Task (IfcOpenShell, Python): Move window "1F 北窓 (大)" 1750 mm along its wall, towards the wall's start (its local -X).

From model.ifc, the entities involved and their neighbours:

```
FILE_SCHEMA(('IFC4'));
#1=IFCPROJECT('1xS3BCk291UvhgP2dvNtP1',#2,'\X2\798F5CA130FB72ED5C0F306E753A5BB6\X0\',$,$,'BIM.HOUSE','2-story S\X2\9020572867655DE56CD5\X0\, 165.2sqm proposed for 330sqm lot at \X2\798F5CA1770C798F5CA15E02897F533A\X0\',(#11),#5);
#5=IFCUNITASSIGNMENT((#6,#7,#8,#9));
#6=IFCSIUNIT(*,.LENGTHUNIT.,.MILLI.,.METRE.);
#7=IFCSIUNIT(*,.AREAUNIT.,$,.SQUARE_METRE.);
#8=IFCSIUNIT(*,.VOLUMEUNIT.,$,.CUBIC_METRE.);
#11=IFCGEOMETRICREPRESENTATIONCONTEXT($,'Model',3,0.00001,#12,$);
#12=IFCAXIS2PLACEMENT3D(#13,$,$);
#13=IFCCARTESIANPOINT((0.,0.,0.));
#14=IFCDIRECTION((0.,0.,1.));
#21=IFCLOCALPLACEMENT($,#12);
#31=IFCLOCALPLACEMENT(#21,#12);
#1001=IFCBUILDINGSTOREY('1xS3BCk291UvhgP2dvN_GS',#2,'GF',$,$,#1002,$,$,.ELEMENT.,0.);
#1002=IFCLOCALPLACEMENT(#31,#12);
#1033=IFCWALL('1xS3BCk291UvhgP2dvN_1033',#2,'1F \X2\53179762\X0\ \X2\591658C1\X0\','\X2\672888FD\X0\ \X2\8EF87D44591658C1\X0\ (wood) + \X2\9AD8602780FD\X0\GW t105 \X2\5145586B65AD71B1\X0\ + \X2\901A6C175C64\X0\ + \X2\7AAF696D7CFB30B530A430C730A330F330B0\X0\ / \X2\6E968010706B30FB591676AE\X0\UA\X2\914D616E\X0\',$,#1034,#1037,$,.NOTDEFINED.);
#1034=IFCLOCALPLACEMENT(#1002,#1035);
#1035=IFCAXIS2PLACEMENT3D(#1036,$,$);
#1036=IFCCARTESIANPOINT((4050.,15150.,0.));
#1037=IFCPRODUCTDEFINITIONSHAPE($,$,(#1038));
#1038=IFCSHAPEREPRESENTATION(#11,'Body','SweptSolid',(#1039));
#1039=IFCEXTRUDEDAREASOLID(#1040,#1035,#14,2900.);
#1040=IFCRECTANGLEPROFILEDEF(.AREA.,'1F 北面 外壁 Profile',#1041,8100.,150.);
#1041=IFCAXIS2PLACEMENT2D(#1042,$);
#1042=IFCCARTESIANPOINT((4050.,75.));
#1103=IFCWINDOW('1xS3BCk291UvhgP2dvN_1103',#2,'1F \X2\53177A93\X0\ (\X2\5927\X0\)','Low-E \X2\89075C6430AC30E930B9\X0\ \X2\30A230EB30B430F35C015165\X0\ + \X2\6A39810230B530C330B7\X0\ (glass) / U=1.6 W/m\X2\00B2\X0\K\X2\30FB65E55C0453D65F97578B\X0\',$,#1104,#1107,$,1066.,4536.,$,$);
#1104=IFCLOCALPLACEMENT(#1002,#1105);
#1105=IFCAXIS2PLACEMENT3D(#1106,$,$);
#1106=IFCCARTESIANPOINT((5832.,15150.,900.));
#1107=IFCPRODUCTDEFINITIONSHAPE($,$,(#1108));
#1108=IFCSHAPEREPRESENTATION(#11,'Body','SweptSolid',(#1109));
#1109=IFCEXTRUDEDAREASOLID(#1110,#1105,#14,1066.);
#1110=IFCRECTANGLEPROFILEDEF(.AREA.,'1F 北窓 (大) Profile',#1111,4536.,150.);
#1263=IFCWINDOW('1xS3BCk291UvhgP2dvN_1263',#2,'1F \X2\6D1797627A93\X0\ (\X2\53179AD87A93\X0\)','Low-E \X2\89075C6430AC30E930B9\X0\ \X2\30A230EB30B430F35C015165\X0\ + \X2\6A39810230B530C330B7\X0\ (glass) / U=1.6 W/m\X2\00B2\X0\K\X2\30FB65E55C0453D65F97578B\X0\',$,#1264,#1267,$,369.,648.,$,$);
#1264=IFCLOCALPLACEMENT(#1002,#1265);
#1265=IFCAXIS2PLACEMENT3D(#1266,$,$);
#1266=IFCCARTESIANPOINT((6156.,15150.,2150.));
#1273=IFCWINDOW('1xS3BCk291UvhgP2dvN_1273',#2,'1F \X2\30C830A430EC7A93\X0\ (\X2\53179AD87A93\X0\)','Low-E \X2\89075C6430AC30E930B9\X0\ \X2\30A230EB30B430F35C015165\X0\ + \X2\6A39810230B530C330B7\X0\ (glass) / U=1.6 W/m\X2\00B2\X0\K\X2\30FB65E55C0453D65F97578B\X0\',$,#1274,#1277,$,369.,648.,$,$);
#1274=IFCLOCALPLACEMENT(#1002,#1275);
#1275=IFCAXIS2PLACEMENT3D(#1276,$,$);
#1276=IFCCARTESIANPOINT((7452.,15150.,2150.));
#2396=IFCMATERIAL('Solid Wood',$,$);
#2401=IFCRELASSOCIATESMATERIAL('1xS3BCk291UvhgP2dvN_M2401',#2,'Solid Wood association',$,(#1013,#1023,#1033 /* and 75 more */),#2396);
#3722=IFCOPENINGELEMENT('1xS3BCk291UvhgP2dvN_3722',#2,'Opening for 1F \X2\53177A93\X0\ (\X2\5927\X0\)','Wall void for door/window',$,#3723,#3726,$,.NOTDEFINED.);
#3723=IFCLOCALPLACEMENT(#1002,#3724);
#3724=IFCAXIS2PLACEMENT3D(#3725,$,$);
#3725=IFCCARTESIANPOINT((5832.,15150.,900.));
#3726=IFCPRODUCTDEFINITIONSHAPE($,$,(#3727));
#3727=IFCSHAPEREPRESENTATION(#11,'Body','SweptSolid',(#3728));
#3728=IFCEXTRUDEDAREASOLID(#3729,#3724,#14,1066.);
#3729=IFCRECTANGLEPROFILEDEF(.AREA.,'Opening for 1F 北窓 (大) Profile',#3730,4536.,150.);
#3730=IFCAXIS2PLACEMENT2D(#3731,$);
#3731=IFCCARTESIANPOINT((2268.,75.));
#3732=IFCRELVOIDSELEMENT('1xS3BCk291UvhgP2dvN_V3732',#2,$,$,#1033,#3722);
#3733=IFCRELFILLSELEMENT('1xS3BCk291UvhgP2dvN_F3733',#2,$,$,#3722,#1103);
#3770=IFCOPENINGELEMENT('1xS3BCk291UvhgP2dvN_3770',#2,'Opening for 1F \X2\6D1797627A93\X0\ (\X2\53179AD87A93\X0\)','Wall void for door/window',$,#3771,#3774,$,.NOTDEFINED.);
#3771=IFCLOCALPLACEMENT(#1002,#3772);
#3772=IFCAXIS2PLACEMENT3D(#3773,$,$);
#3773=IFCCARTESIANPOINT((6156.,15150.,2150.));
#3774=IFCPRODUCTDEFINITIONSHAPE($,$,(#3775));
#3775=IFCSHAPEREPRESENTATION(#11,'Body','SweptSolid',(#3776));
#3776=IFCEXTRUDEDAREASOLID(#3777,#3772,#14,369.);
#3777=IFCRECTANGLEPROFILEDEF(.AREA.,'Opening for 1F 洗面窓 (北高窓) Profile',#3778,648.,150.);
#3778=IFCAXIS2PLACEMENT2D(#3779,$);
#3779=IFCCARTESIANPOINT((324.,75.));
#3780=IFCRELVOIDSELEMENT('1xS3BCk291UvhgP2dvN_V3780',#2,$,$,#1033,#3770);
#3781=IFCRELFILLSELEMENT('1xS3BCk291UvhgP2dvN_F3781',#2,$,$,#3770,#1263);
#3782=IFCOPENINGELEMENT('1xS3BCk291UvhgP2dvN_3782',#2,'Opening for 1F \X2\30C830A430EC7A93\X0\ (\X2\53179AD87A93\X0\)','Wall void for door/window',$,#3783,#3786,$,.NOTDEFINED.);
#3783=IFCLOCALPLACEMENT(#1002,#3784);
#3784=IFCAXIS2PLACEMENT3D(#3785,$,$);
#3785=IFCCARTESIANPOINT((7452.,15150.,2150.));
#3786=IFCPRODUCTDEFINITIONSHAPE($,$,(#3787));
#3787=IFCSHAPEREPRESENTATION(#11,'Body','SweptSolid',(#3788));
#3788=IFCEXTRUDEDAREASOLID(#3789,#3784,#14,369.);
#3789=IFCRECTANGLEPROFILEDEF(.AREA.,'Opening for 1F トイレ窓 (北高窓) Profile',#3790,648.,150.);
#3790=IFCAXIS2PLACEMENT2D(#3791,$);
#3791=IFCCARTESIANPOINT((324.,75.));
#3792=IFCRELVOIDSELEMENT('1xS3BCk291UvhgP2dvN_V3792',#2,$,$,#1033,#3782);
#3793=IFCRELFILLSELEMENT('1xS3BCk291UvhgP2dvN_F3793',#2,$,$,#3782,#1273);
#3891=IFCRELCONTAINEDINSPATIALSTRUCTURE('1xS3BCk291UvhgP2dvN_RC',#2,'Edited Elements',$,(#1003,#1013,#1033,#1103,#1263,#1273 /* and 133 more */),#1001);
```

```python
import ifcopenshell
import ifcopenshell.api.geometry
import ifcopenshell.util.placement

model = ifcopenshell.open("model.ifc")

window = model.by_guid("1xS3BCk291UvhgP2dvN_1103")
opening = window.FillsVoids[0].RelatingOpeningElement
wall = opening.VoidsElements[0].RelatingBuildingElement

wall_matrix = ifcopenshell.util.placement.get_local_placement(wall.ObjectPlacement)
shift = wall_matrix[:3, 0] * -1750.0
before = ifcopenshell.util.placement.get_local_placement(window.ObjectPlacement)[:3, 3].copy()

# The window is not placed relative to its opening, so move both.
for product in (opening, window):
    matrix = ifcopenshell.util.placement.get_local_placement(product.ObjectPlacement)
    matrix[:3, 3] += shift
    ifcopenshell.api.geometry.edit_object_placement(model, product=product, matrix=matrix, is_si=False)

after = ifcopenshell.util.placement.get_local_placement(window.ObjectPlacement)[:3, 3]
print("window moved by", (after - before).round(3) + 0.0)

model.write("model_updated.ifc")
```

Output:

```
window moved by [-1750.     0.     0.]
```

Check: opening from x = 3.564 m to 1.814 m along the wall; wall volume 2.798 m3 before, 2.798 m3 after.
